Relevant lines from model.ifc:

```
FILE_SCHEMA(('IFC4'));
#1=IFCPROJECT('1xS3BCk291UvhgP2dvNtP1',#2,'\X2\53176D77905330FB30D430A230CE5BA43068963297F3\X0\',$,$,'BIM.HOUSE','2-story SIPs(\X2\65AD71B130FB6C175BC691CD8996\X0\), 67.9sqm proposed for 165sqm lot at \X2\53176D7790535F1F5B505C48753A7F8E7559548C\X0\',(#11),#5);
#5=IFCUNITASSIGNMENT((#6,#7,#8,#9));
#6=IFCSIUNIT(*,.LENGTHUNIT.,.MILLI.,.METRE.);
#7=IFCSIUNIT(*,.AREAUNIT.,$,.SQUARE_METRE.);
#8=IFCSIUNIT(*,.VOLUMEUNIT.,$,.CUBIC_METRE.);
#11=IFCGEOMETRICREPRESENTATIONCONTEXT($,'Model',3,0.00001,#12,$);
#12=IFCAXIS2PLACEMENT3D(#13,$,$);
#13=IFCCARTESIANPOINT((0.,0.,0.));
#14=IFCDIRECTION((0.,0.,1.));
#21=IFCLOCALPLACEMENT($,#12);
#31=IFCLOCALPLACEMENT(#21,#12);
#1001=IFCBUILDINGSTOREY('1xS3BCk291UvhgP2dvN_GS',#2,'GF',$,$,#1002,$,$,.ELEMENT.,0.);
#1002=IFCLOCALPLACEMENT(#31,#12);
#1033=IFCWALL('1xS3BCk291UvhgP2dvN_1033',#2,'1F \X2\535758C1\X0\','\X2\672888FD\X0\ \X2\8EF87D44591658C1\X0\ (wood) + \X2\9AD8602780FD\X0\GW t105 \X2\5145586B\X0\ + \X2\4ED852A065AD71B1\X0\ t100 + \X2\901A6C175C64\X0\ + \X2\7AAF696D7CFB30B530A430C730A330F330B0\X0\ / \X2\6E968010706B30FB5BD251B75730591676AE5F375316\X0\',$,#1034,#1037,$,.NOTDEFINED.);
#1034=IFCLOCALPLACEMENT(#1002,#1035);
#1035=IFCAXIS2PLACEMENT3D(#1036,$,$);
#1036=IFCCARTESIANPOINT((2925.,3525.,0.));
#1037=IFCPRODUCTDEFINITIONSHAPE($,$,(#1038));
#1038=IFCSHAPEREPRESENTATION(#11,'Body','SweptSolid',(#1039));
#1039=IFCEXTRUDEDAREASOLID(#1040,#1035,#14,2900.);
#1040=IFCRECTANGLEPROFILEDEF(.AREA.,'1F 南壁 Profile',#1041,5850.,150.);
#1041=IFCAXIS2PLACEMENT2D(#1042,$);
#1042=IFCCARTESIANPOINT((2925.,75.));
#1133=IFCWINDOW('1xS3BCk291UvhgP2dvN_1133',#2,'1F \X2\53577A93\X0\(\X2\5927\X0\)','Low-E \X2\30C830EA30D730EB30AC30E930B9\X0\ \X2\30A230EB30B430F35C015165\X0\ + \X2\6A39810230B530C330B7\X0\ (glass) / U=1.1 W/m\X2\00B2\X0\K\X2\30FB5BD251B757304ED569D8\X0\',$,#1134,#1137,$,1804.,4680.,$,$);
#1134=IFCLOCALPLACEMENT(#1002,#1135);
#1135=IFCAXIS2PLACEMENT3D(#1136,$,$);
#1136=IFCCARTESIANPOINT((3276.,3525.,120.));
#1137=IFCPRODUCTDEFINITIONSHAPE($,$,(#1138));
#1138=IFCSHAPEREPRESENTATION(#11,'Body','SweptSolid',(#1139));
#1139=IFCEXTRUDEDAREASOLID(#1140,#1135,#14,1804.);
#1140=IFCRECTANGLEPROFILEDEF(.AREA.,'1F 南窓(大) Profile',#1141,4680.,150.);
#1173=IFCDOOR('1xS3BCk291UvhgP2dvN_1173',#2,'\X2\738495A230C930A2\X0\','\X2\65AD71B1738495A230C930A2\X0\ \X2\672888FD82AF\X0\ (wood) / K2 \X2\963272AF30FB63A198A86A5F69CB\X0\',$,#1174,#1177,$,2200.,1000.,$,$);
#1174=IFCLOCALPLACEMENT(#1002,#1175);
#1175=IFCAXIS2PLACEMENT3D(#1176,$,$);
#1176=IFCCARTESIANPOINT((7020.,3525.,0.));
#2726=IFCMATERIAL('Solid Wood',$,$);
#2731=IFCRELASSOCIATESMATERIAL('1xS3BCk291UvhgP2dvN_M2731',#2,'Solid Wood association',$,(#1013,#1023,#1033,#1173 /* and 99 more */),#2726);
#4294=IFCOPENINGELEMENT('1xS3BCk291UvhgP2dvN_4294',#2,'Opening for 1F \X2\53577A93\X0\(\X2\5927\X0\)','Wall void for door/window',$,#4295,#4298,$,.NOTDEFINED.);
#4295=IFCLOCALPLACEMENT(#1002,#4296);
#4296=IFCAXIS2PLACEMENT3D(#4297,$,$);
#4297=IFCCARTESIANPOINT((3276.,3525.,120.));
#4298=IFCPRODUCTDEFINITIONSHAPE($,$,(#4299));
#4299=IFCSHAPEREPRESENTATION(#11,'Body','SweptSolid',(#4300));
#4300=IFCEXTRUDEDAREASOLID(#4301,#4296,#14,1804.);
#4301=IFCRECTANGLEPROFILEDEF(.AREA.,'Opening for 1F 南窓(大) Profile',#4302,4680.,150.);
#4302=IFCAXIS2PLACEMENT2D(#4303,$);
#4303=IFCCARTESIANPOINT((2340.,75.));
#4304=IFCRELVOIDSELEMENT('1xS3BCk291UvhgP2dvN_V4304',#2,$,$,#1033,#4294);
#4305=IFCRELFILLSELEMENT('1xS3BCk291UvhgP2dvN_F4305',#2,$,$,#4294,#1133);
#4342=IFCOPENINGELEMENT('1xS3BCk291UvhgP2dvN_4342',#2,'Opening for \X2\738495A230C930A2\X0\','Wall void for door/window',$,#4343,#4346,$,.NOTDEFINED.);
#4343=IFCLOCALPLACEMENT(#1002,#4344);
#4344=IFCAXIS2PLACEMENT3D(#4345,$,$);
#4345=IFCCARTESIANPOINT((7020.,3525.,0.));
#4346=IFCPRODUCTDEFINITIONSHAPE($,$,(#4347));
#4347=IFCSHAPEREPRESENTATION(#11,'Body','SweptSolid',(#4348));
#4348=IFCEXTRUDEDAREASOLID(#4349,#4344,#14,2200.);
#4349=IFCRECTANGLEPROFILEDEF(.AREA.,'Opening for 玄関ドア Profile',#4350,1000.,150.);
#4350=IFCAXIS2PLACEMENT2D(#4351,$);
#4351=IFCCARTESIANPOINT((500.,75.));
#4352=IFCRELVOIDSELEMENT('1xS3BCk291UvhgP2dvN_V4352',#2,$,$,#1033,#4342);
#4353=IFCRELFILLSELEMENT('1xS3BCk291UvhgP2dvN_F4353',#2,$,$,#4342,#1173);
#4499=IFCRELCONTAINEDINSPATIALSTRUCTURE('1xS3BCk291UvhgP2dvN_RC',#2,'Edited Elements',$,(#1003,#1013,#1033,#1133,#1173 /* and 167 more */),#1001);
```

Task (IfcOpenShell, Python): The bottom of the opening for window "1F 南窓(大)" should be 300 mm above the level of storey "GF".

```python
import numpy as np
import ifcopenshell
import ifcopenshell.api.geometry
import ifcopenshell.geom
import ifcopenshell.util.element
import ifcopenshell.util.placement
import ifcopenshell.util.shape
import ifcopenshell.util.unit

model = ifcopenshell.open("model.ifc")
unit_scale = ifcopenshell.util.unit.calculate_unit_scale(model)

window = model.by_id(1133)
opening = window.FillsVoids[0].RelatingOpeningElement
storey = ifcopenshell.util.element.get_container(window, ifc_class="IfcBuildingStorey")
level = ifcopenshell.util.placement.get_local_placement(storey.ObjectPlacement)[2, 3]

# The opening's origin need not be at the sill, so measure its lowest point.
shape = ifcopenshell.geom.create_shape(ifcopenshell.geom.settings(), opening)
bottom = ifcopenshell.util.shape.get_shape_bottom_elevation(shape, shape.geometry) / unit_scale
dz = level + 0.3 / unit_scale - bottom

shift = np.array([0.0, 0.0, dz])
# The window is not placed relative to its opening, so move both.
for product in (opening, window):
    matrix = ifcopenshell.util.placement.get_local_placement(product.ObjectPlacement)
    matrix[:3, 3] += shift
    ifcopenshell.api.geometry.edit_object_placement(model, product=product, matrix=matrix, is_si=False)

print(f"moved by {dz * unit_scale:+.3f} m")

model.write("model_edited.ifc")
```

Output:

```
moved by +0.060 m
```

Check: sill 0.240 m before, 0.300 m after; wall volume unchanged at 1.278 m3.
